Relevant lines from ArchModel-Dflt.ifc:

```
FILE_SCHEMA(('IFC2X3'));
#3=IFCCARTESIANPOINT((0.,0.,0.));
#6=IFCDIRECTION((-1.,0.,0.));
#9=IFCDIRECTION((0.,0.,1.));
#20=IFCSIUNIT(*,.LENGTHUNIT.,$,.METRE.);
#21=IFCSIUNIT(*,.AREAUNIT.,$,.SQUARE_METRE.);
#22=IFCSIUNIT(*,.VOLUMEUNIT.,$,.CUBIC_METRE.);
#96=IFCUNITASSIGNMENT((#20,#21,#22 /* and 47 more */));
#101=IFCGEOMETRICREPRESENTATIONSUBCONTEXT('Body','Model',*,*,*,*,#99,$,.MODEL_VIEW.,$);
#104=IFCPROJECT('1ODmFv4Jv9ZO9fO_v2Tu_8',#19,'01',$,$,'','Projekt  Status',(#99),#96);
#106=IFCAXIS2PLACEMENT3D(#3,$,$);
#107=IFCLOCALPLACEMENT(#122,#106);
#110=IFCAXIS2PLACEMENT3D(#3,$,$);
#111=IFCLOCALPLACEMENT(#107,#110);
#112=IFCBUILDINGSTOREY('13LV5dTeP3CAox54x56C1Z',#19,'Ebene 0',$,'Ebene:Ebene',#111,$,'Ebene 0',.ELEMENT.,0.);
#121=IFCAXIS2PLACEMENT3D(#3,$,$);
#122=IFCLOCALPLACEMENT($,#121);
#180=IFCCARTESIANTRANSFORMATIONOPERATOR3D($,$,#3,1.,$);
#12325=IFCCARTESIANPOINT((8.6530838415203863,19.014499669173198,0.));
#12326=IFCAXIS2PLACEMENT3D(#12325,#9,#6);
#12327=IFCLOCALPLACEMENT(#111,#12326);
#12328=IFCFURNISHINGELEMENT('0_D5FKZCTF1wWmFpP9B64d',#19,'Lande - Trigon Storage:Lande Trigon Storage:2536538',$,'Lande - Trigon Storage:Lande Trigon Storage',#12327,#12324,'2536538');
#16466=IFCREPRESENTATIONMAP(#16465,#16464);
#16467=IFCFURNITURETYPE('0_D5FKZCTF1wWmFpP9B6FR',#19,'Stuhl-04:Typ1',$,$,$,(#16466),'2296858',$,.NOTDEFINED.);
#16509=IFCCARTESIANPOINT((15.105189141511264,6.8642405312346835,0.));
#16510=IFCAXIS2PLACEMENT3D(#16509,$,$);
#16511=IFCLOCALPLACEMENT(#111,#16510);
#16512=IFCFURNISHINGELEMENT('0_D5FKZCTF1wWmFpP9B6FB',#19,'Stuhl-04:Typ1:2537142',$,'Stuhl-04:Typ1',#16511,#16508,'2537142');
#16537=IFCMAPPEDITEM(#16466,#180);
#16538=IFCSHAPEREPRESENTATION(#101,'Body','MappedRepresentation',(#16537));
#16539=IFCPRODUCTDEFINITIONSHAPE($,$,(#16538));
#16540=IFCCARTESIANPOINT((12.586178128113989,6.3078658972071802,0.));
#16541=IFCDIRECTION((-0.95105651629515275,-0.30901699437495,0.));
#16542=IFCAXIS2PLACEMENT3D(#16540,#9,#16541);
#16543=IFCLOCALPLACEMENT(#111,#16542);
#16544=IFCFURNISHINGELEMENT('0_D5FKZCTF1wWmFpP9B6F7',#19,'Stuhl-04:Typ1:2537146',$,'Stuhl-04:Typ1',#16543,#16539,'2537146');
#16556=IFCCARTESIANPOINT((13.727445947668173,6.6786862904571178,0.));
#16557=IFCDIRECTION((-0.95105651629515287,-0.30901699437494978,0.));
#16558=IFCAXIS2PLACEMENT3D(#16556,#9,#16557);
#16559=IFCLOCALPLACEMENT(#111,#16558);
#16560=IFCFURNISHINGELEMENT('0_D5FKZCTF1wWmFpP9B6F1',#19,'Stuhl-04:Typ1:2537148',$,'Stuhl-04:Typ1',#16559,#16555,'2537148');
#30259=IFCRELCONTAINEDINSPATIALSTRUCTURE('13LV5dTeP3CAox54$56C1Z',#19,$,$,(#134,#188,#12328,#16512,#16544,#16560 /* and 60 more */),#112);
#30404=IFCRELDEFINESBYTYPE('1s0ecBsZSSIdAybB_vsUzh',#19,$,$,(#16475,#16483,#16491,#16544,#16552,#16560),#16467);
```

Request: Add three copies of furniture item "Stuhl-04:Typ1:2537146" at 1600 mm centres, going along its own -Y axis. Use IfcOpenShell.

```python
import ifcopenshell
import ifcopenshell.api.geometry
import ifcopenshell.api.root
import ifcopenshell.util.element
import ifcopenshell.util.placement

model = ifcopenshell.open("ArchModel-Dflt.ifc")

source = model.by_guid("0_D5FKZCTF1wWmFpP9B6F7")
base = ifcopenshell.util.placement.get_local_placement(source.ObjectPlacement)
step = -base[:3, 1] * 1.6

for i in range(1, 4):
    copy = ifcopenshell.api.root.copy_class(model, product=source)
    copy.Representation = ifcopenshell.util.element.copy_deep(
        model, source.Representation, exclude=["IfcGeometricRepresentationContext", "IfcRepresentationMap"]
    )
    copy.Name = "Stuhl-04:Typ1"
    copy.Tag = None
    matrix = base.copy()
    matrix[:3, 3] += i * step
    print("added at", matrix[:3, 3].round(3) + 0.0)
    ifcopenshell.api.geometry.edit_object_placement(model, product=copy, matrix=matrix, is_si=False)

model.write("ArchModel-Dflt_v2.ifc")
```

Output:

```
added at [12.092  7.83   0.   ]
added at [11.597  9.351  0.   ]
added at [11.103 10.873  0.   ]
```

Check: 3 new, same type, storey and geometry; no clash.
